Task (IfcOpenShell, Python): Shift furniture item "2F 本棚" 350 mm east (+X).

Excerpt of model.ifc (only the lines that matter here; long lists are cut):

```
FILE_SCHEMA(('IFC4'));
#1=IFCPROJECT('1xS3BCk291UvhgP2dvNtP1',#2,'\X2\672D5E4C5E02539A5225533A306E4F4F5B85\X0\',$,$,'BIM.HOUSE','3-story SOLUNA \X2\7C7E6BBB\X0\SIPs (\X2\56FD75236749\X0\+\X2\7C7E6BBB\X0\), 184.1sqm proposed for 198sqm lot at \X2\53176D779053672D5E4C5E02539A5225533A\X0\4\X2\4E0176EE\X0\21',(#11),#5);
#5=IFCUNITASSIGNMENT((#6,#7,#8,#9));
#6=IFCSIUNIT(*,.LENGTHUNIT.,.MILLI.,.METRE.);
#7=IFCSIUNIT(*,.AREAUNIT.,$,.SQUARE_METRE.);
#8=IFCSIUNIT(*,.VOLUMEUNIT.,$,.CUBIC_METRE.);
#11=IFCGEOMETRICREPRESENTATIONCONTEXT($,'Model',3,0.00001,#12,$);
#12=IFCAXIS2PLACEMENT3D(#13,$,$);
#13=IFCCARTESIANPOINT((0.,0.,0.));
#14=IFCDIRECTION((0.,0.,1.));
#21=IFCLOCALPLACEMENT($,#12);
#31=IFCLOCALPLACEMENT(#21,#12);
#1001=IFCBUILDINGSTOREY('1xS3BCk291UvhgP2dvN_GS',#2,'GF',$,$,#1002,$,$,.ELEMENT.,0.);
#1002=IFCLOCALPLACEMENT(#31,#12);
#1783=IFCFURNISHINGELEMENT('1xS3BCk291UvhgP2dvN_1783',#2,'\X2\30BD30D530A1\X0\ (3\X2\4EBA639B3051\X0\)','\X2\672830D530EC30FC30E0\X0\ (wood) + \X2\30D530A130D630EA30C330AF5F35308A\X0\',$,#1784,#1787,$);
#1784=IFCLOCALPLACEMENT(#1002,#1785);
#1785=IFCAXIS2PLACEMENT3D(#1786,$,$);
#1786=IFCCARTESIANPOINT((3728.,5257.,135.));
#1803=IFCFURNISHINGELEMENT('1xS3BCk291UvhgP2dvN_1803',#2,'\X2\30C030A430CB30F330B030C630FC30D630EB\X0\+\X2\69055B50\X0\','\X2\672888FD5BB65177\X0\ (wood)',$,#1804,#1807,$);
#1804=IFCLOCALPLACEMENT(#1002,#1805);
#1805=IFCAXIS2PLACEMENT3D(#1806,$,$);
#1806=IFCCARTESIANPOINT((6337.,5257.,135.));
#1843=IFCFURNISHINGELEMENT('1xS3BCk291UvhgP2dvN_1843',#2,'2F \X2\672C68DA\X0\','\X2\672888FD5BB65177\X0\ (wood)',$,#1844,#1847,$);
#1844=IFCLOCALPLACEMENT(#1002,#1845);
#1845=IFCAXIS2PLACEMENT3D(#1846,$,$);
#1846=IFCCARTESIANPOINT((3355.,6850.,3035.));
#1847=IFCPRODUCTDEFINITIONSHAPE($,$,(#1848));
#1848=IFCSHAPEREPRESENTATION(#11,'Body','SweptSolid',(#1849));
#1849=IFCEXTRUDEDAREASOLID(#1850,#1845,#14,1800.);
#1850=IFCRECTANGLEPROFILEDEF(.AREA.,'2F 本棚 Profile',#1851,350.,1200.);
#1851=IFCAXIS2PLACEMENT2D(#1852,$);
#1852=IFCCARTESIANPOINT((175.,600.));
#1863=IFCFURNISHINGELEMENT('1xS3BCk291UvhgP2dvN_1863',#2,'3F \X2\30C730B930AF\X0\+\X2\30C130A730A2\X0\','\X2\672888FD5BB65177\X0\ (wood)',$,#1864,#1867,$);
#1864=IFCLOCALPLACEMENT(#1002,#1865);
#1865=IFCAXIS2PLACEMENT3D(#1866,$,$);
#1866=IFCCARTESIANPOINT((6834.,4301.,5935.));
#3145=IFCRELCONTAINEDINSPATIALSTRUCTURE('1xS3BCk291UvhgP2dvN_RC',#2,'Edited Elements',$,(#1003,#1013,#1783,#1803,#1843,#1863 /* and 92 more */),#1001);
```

```python
import ifcopenshell
import ifcopenshell.api.geometry
import ifcopenshell.util.placement
import ifcopenshell.util.unit

model = ifcopenshell.open("model.ifc")
unit_scale = ifcopenshell.util.unit.calculate_unit_scale(model)

item = model.by_id(1843)
matrix = ifcopenshell.util.placement.get_local_placement(item.ObjectPlacement)
matrix[0, 3] += 0.35 / unit_scale
ifcopenshell.api.geometry.edit_object_placement(model, product=item, matrix=matrix, is_si=False)

print(ifcopenshell.util.placement.get_local_placement(item.ObjectPlacement).round(3) + 0.0)

model.write("model_rev.ifc")
```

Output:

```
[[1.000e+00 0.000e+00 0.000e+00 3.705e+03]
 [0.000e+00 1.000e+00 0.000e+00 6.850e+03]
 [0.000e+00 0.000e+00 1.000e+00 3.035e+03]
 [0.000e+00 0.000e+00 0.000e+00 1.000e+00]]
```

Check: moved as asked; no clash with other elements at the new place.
